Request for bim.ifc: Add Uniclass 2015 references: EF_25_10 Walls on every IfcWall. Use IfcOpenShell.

First a look at what the model holds.

```python
import ifcopenshell

model = ifcopenshell.open("bim.ifc")
print(model.schema)
print("classifications:", [c.Name for c in model.by_type("IfcClassification")])
for ifc_class in ("IfcDoor", "IfcRoof", "IfcStair", "IfcWall", "IfcWindow"):
    print(ifc_class, len(model.by_type(ifc_class)))
```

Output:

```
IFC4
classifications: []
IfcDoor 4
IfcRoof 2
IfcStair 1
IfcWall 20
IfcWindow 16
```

```python
import ifcopenshell
import ifcopenshell.api.classification

model = ifcopenshell.open("bim.ifc")

system = ifcopenshell.api.classification.add_classification(model, classification="Uniclass 2015")

codes = {
    "IfcWall": ("EF_25_10", "Walls"),
}
for ifc_class, (code, name) in codes.items():
    products = model.by_type(ifc_class)
    ifcopenshell.api.classification.add_reference(
        model, products=products, classification=system, identification=code, name=name
    )
    print(code, len(products))

model.write("bim_v2.ifc")
```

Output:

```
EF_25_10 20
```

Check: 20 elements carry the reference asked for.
